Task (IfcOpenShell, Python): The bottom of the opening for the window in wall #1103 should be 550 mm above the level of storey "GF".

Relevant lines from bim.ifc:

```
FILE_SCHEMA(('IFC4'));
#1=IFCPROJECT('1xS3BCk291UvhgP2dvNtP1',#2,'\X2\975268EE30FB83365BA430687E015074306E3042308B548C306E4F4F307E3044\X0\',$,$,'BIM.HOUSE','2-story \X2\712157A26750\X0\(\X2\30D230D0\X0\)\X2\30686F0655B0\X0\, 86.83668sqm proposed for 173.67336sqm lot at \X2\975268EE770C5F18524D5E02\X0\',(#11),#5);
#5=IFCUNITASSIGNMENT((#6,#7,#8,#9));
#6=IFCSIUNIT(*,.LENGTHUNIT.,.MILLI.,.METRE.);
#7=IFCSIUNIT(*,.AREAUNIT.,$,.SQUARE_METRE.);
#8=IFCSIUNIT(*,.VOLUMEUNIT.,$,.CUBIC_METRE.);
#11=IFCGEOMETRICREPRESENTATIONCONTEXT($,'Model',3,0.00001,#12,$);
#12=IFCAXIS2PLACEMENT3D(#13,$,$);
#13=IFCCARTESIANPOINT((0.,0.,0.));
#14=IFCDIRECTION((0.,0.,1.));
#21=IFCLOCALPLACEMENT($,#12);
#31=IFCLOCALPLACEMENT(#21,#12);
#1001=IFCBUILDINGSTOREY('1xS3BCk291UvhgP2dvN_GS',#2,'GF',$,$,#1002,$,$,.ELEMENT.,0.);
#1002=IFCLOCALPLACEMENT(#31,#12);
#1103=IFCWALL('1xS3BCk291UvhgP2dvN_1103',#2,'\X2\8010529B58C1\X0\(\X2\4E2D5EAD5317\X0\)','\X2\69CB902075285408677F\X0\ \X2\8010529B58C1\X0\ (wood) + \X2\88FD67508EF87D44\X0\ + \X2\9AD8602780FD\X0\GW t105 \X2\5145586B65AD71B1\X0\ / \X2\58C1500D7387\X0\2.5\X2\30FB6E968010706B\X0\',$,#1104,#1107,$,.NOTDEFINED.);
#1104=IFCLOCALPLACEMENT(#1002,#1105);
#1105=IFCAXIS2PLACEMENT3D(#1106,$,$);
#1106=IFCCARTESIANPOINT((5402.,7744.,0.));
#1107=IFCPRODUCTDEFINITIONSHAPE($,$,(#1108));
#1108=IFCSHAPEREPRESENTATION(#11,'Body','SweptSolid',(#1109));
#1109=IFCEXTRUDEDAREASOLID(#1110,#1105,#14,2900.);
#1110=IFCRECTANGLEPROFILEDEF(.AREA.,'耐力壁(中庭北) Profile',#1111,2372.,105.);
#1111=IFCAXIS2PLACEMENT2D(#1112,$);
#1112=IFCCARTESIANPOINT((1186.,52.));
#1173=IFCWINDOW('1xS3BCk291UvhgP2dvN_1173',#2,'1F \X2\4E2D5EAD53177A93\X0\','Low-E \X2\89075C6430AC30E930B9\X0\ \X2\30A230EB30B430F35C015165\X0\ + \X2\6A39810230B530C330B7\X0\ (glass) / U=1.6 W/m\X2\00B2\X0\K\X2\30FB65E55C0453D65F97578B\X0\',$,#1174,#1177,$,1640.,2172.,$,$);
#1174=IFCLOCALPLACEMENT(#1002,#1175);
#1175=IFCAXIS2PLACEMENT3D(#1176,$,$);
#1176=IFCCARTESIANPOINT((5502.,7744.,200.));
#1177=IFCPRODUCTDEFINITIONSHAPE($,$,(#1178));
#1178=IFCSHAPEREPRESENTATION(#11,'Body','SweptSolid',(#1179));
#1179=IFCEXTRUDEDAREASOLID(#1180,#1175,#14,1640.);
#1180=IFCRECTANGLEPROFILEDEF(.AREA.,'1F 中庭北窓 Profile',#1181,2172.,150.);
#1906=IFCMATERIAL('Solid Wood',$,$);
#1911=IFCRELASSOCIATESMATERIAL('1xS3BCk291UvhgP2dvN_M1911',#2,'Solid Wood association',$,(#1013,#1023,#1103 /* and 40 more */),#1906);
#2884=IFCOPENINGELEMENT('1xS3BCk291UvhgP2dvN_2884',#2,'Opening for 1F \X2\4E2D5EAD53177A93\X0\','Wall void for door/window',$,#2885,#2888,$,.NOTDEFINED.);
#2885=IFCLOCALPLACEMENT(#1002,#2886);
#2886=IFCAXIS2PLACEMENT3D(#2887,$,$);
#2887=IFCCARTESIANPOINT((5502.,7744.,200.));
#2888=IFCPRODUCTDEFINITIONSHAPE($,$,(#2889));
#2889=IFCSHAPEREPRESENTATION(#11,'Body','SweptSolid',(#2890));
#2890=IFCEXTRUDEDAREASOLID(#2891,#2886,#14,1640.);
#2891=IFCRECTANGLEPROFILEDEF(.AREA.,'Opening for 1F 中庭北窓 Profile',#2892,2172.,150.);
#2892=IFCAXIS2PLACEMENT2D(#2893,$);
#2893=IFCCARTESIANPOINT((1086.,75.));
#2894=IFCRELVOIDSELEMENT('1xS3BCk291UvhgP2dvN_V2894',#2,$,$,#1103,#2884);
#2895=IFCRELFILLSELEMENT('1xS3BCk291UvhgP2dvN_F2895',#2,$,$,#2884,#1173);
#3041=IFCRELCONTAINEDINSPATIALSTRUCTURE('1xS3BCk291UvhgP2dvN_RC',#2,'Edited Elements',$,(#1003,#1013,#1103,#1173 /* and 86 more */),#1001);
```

```python
import numpy as np
import ifcopenshell
import ifcopenshell.api.geometry
import ifcopenshell.geom
import ifcopenshell.util.element
import ifcopenshell.util.placement
import ifcopenshell.util.shape
import ifcopenshell.util.unit

model = ifcopenshell.open("bim.ifc")
unit_scale = ifcopenshell.util.unit.calculate_unit_scale(model)

window = model.by_id(1173)
opening = window.FillsVoids[0].RelatingOpeningElement
storey = ifcopenshell.util.element.get_container(window, ifc_class="IfcBuildingStorey")
level = ifcopenshell.util.placement.get_local_placement(storey.ObjectPlacement)[2, 3]

# The opening's origin need not be at the sill, so measure its lowest point.
shape = ifcopenshell.geom.create_shape(ifcopenshell.geom.settings(), opening)
bottom = ifcopenshell.util.shape.get_shape_bottom_elevation(shape, shape.geometry) / unit_scale
dz = level + 0.55 / unit_scale - bottom

shift = np.array([0.0, 0.0, dz])
# The window is not placed relative to its opening, so move both.
for product in (opening, window):
    matrix = ifcopenshell.util.placement.get_local_placement(product.ObjectPlacement)
    matrix[:3, 3] += shift
    ifcopenshell.api.geometry.edit_object_placement(model, product=product, matrix=matrix, is_si=False)

print(f"moved by {dz * unit_scale:+.3f} m")

model.write("bim_edited.ifc")
```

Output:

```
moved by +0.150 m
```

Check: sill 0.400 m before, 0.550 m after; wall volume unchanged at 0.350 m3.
